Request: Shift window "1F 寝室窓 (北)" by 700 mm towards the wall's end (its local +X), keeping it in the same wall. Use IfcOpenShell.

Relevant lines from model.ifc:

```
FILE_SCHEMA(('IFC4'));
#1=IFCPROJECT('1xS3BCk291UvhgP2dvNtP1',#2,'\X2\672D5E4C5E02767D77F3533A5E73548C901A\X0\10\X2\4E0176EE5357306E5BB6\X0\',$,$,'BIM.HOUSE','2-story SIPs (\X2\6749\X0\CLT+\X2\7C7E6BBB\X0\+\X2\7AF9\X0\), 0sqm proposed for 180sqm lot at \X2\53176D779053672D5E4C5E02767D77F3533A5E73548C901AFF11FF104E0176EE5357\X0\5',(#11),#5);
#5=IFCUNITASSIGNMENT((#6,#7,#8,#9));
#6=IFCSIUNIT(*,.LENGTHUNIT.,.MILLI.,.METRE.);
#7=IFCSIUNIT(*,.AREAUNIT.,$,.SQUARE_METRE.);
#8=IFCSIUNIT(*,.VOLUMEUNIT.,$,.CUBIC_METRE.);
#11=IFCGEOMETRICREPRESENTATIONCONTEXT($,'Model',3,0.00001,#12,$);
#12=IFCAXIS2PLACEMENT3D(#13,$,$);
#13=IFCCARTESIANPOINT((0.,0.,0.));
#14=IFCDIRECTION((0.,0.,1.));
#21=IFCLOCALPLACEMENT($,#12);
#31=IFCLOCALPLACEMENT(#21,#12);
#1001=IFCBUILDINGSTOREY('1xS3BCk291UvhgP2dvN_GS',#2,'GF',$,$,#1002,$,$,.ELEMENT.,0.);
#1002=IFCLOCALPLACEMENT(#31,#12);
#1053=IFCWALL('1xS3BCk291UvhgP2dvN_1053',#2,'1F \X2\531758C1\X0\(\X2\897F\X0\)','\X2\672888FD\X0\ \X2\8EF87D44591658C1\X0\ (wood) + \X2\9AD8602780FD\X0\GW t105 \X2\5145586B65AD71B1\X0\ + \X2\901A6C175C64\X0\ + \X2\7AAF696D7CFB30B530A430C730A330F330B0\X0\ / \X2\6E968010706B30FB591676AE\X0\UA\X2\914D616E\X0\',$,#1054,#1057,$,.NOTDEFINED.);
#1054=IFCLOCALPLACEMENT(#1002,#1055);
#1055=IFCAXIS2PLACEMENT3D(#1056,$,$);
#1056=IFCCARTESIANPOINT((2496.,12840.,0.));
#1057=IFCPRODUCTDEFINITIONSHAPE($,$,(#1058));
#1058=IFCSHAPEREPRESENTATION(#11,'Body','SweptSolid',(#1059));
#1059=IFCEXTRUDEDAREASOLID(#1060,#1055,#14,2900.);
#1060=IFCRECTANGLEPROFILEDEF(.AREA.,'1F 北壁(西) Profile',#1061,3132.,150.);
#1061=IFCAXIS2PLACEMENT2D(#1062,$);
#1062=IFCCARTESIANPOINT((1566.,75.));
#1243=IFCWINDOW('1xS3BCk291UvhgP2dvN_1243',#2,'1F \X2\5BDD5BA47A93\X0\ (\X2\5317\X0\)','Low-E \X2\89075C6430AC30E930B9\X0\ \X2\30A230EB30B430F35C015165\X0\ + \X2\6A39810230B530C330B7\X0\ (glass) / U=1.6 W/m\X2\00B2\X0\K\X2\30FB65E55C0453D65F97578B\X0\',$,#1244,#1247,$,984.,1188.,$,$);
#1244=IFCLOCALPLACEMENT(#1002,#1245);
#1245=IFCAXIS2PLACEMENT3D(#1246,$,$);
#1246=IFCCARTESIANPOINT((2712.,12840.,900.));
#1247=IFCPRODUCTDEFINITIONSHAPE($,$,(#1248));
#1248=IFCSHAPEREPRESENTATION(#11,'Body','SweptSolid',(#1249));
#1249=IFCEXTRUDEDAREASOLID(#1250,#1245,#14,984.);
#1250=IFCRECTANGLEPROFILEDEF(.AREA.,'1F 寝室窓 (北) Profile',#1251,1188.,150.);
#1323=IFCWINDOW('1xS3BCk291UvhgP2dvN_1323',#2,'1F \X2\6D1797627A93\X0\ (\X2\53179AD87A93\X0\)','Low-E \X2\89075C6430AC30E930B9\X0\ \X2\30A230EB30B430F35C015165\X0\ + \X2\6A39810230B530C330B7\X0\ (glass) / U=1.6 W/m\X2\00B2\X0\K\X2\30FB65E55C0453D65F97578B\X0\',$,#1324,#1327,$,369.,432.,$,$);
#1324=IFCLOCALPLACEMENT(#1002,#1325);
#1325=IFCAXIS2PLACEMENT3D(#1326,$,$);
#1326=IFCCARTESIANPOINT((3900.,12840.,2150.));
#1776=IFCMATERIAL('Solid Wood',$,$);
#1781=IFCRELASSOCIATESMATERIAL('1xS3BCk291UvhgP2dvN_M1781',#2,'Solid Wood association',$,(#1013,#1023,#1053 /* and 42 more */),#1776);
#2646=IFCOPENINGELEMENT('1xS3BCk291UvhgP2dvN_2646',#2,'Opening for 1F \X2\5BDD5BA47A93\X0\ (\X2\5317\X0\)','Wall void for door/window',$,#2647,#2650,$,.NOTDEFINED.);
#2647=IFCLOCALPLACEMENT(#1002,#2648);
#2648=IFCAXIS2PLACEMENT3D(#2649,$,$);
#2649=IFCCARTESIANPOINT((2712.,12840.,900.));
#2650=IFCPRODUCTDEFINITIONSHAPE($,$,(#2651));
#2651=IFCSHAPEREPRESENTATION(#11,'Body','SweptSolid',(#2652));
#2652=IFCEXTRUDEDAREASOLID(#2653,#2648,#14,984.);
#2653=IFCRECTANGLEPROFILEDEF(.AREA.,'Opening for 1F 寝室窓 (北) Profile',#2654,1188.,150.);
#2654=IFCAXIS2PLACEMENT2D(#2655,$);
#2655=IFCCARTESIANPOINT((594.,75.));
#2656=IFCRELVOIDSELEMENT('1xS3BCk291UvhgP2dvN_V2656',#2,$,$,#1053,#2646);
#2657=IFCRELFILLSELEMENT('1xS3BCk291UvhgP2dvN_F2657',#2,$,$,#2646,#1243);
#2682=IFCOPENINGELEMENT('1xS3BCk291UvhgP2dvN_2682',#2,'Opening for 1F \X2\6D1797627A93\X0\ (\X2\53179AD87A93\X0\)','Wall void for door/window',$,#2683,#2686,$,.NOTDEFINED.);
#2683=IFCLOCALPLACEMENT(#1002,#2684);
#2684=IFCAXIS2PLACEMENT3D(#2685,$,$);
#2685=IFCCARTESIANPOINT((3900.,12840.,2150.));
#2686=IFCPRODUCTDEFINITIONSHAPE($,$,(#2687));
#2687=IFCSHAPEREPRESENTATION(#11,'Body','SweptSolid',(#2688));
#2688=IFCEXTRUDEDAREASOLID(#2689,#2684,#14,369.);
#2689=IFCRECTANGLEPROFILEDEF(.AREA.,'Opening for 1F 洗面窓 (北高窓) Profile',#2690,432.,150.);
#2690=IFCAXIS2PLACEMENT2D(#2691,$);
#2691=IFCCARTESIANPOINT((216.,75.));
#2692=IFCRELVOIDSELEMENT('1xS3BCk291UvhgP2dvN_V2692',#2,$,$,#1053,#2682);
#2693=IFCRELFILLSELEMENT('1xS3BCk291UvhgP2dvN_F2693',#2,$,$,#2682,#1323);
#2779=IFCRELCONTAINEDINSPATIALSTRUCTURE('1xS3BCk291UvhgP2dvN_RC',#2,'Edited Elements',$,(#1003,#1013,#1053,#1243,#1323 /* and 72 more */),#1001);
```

```python
import ifcopenshell
import ifcopenshell.api.geometry
import ifcopenshell.util.placement

model = ifcopenshell.open("model.ifc")

window = model.by_guid("1xS3BCk291UvhgP2dvN_1243")
opening = window.FillsVoids[0].RelatingOpeningElement
wall = opening.VoidsElements[0].RelatingBuildingElement

wall_matrix = ifcopenshell.util.placement.get_local_placement(wall.ObjectPlacement)
shift = wall_matrix[:3, 0] * 700.0
before = ifcopenshell.util.placement.get_local_placement(window.ObjectPlacement)[:3, 3].copy()

# The window is not placed relative to its opening, so move both.
for product in (opening, window):
    matrix = ifcopenshell.util.placement.get_local_placement(product.ObjectPlacement)
    matrix[:3, 3] += shift
    ifcopenshell.api.geometry.edit_object_placement(model, product=product, matrix=matrix, is_si=False)

after = ifcopenshell.util.placement.get_local_placement(window.ObjectPlacement)[:3, 3]
print("window moved by", (after - before).round(3) + 0.0)

model.write("model_rev.ifc")
```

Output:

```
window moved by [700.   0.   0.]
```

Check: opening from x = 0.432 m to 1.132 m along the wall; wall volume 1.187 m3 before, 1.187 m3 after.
